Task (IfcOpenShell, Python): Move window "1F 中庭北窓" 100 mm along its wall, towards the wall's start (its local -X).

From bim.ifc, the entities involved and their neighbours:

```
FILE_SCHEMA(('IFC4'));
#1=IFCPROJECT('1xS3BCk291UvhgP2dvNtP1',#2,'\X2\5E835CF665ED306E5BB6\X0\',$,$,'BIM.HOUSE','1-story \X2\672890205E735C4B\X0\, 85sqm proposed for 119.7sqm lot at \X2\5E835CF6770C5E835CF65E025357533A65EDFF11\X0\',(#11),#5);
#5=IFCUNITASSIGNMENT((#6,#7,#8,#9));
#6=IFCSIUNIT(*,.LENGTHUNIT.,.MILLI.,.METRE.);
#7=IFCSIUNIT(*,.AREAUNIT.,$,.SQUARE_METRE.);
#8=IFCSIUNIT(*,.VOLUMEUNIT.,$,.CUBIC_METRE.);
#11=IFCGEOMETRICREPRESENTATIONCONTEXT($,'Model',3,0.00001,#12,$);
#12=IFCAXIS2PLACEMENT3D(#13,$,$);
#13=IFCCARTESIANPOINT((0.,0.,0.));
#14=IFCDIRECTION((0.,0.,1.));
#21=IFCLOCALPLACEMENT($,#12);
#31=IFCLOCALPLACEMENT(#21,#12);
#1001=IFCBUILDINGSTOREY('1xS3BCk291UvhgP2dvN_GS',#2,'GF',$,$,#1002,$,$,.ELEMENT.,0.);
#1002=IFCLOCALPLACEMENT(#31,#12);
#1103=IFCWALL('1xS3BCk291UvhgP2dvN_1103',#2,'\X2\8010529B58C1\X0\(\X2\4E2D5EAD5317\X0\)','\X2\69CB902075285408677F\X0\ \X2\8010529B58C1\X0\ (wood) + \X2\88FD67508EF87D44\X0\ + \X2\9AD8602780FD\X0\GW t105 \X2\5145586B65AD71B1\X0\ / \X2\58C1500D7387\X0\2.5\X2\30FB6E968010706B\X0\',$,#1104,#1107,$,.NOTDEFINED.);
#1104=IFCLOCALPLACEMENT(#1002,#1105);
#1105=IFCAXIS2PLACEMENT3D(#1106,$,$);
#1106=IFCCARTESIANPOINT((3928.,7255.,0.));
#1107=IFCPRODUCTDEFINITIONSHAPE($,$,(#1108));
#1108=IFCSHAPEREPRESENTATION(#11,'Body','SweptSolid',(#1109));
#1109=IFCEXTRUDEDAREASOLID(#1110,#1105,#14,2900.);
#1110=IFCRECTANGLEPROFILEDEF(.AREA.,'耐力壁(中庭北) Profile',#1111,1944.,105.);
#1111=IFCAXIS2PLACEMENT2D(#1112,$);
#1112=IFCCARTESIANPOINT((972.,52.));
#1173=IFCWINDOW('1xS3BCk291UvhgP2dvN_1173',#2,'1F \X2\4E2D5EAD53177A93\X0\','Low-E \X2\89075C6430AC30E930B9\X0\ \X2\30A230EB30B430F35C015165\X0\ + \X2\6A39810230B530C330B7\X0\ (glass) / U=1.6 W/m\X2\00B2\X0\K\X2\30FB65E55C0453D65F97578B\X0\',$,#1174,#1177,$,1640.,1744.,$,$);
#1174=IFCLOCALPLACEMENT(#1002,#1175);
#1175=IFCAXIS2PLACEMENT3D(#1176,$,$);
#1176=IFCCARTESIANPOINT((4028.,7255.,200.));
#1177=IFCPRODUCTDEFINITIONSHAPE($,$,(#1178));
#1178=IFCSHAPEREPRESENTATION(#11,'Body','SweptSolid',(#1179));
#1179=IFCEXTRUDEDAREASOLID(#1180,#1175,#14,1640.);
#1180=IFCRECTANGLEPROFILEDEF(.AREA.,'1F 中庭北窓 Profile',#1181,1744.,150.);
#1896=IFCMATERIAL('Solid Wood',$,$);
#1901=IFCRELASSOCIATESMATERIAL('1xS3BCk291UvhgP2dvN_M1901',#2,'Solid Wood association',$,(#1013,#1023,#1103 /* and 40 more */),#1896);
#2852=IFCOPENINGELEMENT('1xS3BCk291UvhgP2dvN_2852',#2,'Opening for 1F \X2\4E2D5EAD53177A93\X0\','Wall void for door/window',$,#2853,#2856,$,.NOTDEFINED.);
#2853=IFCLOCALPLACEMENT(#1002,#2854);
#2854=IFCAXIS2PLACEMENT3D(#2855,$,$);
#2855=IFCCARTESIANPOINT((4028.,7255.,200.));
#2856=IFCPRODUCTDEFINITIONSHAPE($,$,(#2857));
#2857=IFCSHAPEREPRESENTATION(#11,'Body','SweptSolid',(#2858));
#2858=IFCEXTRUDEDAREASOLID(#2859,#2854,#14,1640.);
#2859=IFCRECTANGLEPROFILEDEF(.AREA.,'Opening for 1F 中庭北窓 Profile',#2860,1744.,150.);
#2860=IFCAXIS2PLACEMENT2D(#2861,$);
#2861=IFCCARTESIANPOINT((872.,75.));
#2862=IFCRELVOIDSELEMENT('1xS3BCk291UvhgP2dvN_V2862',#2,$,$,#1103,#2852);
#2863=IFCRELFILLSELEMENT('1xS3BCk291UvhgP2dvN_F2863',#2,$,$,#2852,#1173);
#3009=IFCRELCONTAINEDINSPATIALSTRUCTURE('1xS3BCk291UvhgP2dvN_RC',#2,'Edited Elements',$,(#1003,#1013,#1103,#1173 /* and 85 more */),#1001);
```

```python
import ifcopenshell
import ifcopenshell.api.geometry
import ifcopenshell.util.placement

model = ifcopenshell.open("bim.ifc")

window = model.by_guid("1xS3BCk291UvhgP2dvN_1173")
opening = window.FillsVoids[0].RelatingOpeningElement
wall = opening.VoidsElements[0].RelatingBuildingElement

wall_matrix = ifcopenshell.util.placement.get_local_placement(wall.ObjectPlacement)
shift = wall_matrix[:3, 0] * -100.0
before = ifcopenshell.util.placement.get_local_placement(window.ObjectPlacement)[:3, 3].copy()

# The window is not placed relative to its opening, so move both.
for product in (opening, window):
    matrix = ifcopenshell.util.placement.get_local_placement(product.ObjectPlacement)
    matrix[:3, 3] += shift
    ifcopenshell.api.geometry.edit_object_placement(model, product=product, matrix=matrix, is_si=False)

after = ifcopenshell.util.placement.get_local_placement(window.ObjectPlacement)[:3, 3]
print("window moved by", (after - before).round(3) + 0.0)

model.write("bim-out.ifc")
```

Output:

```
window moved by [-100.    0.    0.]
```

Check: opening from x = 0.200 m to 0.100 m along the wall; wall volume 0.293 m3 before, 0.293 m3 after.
